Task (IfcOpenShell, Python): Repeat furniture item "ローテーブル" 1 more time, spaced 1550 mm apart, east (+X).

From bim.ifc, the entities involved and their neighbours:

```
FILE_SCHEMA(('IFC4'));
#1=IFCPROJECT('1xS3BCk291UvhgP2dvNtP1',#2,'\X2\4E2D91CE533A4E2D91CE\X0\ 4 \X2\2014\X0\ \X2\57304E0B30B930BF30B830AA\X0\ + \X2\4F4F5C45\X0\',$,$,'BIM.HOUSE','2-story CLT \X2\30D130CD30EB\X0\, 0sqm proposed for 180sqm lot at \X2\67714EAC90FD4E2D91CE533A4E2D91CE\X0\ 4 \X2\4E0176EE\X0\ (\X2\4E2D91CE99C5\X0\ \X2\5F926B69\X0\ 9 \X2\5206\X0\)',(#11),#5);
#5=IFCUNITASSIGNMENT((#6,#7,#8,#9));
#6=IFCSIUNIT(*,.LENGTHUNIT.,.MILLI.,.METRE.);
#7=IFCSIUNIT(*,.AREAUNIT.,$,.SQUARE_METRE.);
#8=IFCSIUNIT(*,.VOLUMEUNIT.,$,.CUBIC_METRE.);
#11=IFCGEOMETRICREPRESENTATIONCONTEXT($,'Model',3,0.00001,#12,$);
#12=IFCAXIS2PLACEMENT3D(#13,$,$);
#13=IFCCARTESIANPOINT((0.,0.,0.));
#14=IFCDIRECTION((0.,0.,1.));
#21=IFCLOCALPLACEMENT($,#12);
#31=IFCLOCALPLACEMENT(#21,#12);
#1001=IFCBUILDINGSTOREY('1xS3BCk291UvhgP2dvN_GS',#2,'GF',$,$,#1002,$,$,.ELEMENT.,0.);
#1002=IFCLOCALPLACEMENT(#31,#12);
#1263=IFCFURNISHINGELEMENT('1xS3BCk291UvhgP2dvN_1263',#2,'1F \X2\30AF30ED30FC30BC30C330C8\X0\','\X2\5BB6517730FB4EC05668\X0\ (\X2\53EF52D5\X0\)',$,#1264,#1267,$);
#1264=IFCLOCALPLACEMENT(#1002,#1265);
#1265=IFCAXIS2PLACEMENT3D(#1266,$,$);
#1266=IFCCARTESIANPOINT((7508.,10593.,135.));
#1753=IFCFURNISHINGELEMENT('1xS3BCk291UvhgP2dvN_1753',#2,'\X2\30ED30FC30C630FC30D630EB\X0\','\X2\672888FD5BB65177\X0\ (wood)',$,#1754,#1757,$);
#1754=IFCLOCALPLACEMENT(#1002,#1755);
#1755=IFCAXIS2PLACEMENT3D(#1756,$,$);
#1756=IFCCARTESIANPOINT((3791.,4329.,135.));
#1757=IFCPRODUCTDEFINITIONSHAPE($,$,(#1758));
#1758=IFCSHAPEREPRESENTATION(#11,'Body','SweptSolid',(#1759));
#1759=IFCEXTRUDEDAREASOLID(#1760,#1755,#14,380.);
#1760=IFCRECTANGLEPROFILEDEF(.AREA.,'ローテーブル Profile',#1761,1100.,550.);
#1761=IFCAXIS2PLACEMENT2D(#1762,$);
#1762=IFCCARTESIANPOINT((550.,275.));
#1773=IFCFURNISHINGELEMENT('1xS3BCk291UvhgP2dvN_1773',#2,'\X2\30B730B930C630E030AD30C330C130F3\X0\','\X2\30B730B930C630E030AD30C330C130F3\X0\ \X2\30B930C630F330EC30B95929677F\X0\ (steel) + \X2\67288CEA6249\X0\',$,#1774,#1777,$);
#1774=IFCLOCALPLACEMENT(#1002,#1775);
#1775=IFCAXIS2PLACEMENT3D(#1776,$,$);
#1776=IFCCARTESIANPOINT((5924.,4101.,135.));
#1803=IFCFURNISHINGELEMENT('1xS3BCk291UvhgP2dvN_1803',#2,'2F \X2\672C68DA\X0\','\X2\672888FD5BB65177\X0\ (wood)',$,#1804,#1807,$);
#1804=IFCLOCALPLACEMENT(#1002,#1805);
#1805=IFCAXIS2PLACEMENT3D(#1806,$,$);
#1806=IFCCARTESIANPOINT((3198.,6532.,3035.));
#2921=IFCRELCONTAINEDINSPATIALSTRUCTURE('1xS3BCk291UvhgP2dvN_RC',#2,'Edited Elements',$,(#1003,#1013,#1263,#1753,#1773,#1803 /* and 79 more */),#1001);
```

```python
import numpy as np
import ifcopenshell
import ifcopenshell.api.geometry
import ifcopenshell.api.root
import ifcopenshell.util.element
import ifcopenshell.util.placement
import ifcopenshell.util.unit

model = ifcopenshell.open("bim.ifc")
unit_scale = ifcopenshell.util.unit.calculate_unit_scale(model)


def reuse_history(source, copy):
    """copy_class also copies each property set's owner history, people and application; keep the originals."""
    for rel in copy.IsDefinedBy:
        if rel.is_a("IfcRelDefinesByProperties") and (history := rel.RelatingPropertyDefinition.OwnerHistory):
            rel.RelatingPropertyDefinition.OwnerHistory = source.OwnerHistory
            ifcopenshell.util.element.remove_deep2(model, history)


source = model.by_guid("1xS3BCk291UvhgP2dvN_1753")
base = ifcopenshell.util.placement.get_local_placement(source.ObjectPlacement)
step = np.array([1.0, 0.0, 0.0]) * 1.55 / unit_scale

for i in range(1, 2):
    copy = ifcopenshell.api.root.copy_class(model, product=source)
    copy.Representation = ifcopenshell.util.element.copy_deep(
        model, source.Representation, exclude=["IfcGeometricRepresentationContext", "IfcRepresentationMap"]
    )
    reuse_history(source, copy)
    matrix = base.copy()
    matrix[:3, 3] += i * step
    print("added at", matrix[:3, 3].round(3) + 0.0)
    ifcopenshell.api.geometry.edit_object_placement(model, product=copy, matrix=matrix, is_si=False)

model.write("bim_updated.ifc")
```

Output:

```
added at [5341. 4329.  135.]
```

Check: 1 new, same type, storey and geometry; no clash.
